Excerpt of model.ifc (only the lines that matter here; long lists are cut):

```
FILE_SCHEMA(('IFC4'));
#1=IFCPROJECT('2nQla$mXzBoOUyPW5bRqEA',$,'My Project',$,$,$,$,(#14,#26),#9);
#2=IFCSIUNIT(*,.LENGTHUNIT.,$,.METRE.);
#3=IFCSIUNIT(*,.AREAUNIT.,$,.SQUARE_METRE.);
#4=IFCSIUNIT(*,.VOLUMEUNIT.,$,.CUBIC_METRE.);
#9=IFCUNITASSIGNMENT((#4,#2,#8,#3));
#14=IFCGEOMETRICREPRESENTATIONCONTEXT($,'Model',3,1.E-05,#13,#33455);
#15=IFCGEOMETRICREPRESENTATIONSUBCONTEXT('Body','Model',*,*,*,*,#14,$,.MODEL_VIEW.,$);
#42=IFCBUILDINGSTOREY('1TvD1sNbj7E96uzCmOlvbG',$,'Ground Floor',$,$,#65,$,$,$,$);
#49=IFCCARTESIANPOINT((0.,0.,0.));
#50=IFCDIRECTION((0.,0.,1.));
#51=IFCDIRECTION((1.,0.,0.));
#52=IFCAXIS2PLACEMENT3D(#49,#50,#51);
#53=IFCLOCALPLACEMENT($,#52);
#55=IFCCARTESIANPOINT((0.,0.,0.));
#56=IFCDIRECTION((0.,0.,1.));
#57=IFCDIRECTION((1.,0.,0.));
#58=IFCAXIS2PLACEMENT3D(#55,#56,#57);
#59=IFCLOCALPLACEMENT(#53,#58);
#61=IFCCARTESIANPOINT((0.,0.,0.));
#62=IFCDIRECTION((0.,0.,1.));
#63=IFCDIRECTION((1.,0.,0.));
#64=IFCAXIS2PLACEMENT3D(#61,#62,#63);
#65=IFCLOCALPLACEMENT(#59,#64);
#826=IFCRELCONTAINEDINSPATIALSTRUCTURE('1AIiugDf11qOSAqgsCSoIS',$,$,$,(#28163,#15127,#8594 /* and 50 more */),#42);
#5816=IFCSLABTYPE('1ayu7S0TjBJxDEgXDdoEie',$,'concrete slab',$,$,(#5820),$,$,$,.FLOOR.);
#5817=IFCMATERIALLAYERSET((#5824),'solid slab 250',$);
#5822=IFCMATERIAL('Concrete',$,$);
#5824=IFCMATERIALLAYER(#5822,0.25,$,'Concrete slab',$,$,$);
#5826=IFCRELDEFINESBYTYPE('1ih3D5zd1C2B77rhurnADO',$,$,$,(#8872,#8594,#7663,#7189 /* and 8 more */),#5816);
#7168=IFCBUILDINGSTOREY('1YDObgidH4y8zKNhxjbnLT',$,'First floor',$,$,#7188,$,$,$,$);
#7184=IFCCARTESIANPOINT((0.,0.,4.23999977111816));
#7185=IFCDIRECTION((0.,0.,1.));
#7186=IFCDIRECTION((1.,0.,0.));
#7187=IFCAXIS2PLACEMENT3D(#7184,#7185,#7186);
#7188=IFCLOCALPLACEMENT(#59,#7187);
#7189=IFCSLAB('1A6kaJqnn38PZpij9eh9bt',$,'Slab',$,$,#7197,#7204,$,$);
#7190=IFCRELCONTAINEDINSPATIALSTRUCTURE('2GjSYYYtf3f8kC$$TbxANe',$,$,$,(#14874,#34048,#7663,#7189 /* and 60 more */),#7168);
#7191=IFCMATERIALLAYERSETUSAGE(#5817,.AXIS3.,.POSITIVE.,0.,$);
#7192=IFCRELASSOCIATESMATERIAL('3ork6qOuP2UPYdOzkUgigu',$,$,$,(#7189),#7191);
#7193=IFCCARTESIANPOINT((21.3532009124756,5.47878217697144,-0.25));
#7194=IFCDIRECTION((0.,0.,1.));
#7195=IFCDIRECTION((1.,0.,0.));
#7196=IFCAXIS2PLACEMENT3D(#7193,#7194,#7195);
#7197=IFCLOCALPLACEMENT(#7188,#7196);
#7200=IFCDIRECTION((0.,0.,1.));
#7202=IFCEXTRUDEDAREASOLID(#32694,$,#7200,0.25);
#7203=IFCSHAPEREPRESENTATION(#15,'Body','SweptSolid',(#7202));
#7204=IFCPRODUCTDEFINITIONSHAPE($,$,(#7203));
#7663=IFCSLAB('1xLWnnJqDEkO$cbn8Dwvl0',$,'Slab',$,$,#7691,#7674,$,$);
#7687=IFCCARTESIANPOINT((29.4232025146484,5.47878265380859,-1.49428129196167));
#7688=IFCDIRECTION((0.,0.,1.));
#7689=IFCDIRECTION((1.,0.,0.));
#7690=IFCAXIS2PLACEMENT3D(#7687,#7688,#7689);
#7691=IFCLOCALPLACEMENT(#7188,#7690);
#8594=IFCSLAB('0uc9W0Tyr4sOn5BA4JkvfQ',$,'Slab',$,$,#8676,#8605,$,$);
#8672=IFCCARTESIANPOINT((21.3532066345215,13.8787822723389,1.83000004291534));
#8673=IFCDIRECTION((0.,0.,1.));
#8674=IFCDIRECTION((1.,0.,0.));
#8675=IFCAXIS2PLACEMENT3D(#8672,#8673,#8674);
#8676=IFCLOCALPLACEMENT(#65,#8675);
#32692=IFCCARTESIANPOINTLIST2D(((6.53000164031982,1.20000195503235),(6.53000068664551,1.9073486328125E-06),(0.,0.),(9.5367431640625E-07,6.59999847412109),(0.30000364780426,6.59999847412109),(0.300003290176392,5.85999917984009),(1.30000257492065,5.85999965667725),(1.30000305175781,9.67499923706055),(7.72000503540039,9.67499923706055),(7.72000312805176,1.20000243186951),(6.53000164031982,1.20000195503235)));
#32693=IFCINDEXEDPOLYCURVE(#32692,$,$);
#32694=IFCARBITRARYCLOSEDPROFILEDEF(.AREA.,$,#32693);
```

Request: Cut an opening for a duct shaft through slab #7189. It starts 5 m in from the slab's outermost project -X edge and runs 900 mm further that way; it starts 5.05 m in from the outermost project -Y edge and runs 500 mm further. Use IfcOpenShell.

```python
import numpy as np
import ifcopenshell
import ifcopenshell.api.feature
import ifcopenshell.api.geometry
import ifcopenshell.api.root
import ifcopenshell.geom
import ifcopenshell.util.placement
import ifcopenshell.util.representation
import ifcopenshell.util.shape
import ifcopenshell.util.unit

model = ifcopenshell.open("model.ifc")
unit_scale = ifcopenshell.util.unit.calculate_unit_scale(model)
settings = ifcopenshell.geom.settings()


def volume(element):
    """Net volume in cubic metres, openings subtracted."""
    shape = ifcopenshell.geom.create_shape(settings, element)
    return ifcopenshell.util.shape.get_volume(shape.geometry)


slab = model.by_guid("1A6kaJqnn38PZpij9eh9bt")
before = volume(slab)

# Extent in the slab's own axes, in metres. The edges named are its -X and -Y sides.
slab_shape = ifcopenshell.geom.create_shape(settings, slab)
vertices = ifcopenshell.util.shape.get_vertices(slab_shape.geometry)
x_min, y_min, bottom = vertices.min(axis=0)
top = vertices[:, 2].max()

opening = ifcopenshell.api.root.create_entity(model, ifc_class="IfcOpeningElement", name="Duct shaft opening", predefined_type="OPENING")
context = ifcopenshell.util.representation.get_context(model, "Model", "Body", "MODEL_VIEW")
width, depth = 0.9, 0.5
outline = [(0.0, 0.0), (width, 0.0), (width, depth), (0.0, depth), (0.0, 0.0)]
# Overshoot both faces by 50 mm so the cut is clean.
shape = ifcopenshell.api.geometry.add_slab_representation(
    model, context=context, depth=top - bottom + 0.1, polyline=outline
)
ifcopenshell.api.geometry.assign_representation(model, product=opening, representation=shape)

matrix = ifcopenshell.util.placement.get_local_placement(slab.ObjectPlacement)
matrix[:, 3] = matrix @ np.append(np.array([x_min + 5, y_min + 5.05, bottom - 0.05]) / unit_scale, 1.0)
ifcopenshell.api.geometry.edit_object_placement(model, product=opening, matrix=matrix, is_si=False)
ifcopenshell.api.feature.add_feature(model, feature=opening, element=slab)

after = volume(slab)

print(f"slab volume {before:.3f} -> {after:.3f} m3")

model.write("model-out.ifc")
```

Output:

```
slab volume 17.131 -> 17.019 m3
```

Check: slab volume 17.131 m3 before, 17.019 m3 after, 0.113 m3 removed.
